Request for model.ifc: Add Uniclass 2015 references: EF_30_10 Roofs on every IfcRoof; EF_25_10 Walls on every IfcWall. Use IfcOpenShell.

First a look at what the model holds.

```python
import ifcopenshell

model = ifcopenshell.open("model.ifc")
print(model.schema)
print("classifications:", [c.Name for c in model.by_type("IfcClassification")])
for ifc_class in ("IfcDoor", "IfcRoof", "IfcStair", "IfcWall", "IfcWindow"):
    print(ifc_class, len(model.by_type(ifc_class)))
```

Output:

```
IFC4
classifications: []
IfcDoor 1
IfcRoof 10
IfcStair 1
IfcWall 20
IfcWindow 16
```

```python
import ifcopenshell
import ifcopenshell.api.classification

model = ifcopenshell.open("model.ifc")

system = ifcopenshell.api.classification.add_classification(model, classification="Uniclass 2015")

codes = {
    "IfcRoof": ("EF_30_10", "Roofs"),
    "IfcWall": ("EF_25_10", "Walls"),
}
for ifc_class, (code, name) in codes.items():
    products = model.by_type(ifc_class)
    ifcopenshell.api.classification.add_reference(
        model, products=products, classification=system, identification=code, name=name
    )
    print(code, len(products))

model.write("model_v2.ifc")
```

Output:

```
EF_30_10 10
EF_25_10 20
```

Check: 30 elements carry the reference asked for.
